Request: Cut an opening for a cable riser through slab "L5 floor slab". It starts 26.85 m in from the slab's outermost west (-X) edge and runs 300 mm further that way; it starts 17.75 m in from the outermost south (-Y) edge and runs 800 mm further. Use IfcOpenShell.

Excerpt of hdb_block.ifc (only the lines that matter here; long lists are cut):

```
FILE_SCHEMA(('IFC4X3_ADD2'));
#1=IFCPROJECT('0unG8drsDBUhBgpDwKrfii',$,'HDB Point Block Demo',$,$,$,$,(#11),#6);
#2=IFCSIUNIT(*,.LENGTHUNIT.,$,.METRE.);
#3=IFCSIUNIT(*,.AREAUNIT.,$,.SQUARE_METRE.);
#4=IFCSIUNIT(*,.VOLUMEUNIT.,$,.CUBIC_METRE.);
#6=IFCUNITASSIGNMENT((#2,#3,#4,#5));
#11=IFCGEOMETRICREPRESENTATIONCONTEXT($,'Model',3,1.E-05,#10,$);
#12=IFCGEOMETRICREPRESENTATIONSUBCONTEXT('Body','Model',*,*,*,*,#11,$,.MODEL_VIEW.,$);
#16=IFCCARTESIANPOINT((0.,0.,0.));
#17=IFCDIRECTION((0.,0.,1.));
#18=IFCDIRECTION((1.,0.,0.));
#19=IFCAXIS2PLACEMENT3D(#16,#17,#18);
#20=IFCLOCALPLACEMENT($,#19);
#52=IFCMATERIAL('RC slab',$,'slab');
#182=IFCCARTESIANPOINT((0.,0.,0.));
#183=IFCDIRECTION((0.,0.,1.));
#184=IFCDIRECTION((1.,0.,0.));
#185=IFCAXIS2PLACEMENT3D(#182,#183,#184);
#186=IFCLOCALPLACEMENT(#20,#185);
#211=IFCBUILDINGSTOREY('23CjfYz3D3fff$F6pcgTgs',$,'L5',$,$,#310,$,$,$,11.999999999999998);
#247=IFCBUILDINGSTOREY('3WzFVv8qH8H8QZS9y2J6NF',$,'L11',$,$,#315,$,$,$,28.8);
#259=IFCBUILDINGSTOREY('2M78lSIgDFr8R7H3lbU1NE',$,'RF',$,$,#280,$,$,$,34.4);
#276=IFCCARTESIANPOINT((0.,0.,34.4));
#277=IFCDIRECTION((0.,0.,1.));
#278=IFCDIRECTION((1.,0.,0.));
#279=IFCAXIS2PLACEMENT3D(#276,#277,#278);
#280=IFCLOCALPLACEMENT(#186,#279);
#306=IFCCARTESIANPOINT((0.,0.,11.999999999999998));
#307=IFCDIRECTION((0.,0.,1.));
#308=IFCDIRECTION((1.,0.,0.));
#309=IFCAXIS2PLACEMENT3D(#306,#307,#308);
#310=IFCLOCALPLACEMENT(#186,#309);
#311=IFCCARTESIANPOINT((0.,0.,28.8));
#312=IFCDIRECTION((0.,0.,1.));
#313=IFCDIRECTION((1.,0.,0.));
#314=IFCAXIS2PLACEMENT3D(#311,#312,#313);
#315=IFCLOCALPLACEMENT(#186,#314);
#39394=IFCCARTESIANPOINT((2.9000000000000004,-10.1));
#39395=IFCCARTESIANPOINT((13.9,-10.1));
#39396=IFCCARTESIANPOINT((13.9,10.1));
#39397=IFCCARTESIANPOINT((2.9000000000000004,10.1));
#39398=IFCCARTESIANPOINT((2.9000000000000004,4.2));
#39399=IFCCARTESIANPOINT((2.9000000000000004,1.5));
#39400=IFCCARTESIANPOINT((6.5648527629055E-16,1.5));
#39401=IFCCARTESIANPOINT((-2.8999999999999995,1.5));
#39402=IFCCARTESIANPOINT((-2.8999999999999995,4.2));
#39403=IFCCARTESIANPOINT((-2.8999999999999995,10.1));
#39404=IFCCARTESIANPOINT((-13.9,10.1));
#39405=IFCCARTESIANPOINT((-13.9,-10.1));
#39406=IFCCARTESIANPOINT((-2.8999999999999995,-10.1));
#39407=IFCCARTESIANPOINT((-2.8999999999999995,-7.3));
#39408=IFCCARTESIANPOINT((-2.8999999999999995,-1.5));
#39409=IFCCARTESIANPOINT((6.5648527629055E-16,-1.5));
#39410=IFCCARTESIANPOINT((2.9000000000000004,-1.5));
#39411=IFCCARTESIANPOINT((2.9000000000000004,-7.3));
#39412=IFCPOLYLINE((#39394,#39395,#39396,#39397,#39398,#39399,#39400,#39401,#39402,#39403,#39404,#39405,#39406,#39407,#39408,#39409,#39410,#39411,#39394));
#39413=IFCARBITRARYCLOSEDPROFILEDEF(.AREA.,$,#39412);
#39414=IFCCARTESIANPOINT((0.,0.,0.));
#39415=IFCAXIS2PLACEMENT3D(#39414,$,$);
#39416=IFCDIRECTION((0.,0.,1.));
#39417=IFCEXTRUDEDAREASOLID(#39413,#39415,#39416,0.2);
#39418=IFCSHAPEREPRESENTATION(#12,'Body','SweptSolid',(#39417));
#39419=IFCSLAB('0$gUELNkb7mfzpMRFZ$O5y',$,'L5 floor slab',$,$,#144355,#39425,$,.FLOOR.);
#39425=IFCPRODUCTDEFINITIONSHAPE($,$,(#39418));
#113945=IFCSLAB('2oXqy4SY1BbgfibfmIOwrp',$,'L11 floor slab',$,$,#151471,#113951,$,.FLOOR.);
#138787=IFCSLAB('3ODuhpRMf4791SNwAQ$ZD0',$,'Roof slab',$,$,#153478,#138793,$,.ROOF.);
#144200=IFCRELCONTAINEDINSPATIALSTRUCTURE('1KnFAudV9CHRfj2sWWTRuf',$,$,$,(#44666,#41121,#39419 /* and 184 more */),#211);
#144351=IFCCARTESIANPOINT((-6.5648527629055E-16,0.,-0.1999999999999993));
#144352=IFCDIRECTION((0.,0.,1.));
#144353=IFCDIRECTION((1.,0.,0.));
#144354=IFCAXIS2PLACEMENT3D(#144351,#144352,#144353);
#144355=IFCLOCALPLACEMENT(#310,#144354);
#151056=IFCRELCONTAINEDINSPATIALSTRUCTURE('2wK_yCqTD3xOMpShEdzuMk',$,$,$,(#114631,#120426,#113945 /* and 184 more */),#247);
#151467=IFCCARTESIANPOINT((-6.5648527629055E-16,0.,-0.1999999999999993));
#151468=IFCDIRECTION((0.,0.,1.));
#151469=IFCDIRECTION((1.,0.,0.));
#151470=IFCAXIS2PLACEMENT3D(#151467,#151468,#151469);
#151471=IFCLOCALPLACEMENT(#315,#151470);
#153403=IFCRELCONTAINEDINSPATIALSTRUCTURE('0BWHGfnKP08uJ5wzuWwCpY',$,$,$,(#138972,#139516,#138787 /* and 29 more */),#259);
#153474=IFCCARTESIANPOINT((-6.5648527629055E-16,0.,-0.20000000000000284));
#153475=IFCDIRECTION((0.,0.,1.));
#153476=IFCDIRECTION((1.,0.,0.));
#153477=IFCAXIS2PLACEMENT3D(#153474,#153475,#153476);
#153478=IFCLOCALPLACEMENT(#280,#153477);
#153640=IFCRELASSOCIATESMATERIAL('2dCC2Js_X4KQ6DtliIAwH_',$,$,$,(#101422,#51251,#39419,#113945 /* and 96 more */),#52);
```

```python
import numpy as np
import ifcopenshell
import ifcopenshell.api.feature
import ifcopenshell.api.geometry
import ifcopenshell.api.root
import ifcopenshell.geom
import ifcopenshell.util.placement
import ifcopenshell.util.representation
import ifcopenshell.util.shape
import ifcopenshell.util.unit

model = ifcopenshell.open("hdb_block.ifc")
unit_scale = ifcopenshell.util.unit.calculate_unit_scale(model)
settings = ifcopenshell.geom.settings()


def volume(element):
    """Net volume in cubic metres, openings subtracted."""
    shape = ifcopenshell.geom.create_shape(settings, element)
    return ifcopenshell.util.shape.get_volume(shape.geometry)


slab = model.by_guid("0$gUELNkb7mfzpMRFZ$O5y")
before = volume(slab)

# Extent in the slab's own axes, in metres. The edges named are its -X and -Y sides.
slab_shape = ifcopenshell.geom.create_shape(settings, slab)
vertices = ifcopenshell.util.shape.get_vertices(slab_shape.geometry)
x_min, y_min, bottom = vertices.min(axis=0)
top = vertices[:, 2].max()

opening = ifcopenshell.api.root.create_entity(model, ifc_class="IfcOpeningElement", name="Cable riser opening", predefined_type="OPENING")
context = ifcopenshell.util.representation.get_context(model, "Model", "Body", "MODEL_VIEW")
width, depth = 0.3, 0.8
outline = [(0.0, 0.0), (width, 0.0), (width, depth), (0.0, depth), (0.0, 0.0)]
# Overshoot both faces by 50 mm so the cut is clean.
shape = ifcopenshell.api.geometry.add_slab_representation(
    model, context=context, depth=top - bottom + 0.1, polyline=outline
)
ifcopenshell.api.geometry.assign_representation(model, product=opening, representation=shape)

matrix = ifcopenshell.util.placement.get_local_placement(slab.ObjectPlacement)
matrix[:, 3] = matrix @ np.append(np.array([x_min + 26.85, y_min + 17.75, bottom - 0.05]) / unit_scale, 1.0)
ifcopenshell.api.geometry.edit_object_placement(model, product=opening, matrix=matrix, is_si=False)
ifcopenshell.api.feature.add_feature(model, feature=opening, element=slab)

after = volume(slab)

print(f"slab volume {before:.3f} -> {after:.3f} m3")

model.write("hdb_block_v2.ifc")
```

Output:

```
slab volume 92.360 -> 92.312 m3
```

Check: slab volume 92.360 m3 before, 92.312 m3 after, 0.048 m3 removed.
